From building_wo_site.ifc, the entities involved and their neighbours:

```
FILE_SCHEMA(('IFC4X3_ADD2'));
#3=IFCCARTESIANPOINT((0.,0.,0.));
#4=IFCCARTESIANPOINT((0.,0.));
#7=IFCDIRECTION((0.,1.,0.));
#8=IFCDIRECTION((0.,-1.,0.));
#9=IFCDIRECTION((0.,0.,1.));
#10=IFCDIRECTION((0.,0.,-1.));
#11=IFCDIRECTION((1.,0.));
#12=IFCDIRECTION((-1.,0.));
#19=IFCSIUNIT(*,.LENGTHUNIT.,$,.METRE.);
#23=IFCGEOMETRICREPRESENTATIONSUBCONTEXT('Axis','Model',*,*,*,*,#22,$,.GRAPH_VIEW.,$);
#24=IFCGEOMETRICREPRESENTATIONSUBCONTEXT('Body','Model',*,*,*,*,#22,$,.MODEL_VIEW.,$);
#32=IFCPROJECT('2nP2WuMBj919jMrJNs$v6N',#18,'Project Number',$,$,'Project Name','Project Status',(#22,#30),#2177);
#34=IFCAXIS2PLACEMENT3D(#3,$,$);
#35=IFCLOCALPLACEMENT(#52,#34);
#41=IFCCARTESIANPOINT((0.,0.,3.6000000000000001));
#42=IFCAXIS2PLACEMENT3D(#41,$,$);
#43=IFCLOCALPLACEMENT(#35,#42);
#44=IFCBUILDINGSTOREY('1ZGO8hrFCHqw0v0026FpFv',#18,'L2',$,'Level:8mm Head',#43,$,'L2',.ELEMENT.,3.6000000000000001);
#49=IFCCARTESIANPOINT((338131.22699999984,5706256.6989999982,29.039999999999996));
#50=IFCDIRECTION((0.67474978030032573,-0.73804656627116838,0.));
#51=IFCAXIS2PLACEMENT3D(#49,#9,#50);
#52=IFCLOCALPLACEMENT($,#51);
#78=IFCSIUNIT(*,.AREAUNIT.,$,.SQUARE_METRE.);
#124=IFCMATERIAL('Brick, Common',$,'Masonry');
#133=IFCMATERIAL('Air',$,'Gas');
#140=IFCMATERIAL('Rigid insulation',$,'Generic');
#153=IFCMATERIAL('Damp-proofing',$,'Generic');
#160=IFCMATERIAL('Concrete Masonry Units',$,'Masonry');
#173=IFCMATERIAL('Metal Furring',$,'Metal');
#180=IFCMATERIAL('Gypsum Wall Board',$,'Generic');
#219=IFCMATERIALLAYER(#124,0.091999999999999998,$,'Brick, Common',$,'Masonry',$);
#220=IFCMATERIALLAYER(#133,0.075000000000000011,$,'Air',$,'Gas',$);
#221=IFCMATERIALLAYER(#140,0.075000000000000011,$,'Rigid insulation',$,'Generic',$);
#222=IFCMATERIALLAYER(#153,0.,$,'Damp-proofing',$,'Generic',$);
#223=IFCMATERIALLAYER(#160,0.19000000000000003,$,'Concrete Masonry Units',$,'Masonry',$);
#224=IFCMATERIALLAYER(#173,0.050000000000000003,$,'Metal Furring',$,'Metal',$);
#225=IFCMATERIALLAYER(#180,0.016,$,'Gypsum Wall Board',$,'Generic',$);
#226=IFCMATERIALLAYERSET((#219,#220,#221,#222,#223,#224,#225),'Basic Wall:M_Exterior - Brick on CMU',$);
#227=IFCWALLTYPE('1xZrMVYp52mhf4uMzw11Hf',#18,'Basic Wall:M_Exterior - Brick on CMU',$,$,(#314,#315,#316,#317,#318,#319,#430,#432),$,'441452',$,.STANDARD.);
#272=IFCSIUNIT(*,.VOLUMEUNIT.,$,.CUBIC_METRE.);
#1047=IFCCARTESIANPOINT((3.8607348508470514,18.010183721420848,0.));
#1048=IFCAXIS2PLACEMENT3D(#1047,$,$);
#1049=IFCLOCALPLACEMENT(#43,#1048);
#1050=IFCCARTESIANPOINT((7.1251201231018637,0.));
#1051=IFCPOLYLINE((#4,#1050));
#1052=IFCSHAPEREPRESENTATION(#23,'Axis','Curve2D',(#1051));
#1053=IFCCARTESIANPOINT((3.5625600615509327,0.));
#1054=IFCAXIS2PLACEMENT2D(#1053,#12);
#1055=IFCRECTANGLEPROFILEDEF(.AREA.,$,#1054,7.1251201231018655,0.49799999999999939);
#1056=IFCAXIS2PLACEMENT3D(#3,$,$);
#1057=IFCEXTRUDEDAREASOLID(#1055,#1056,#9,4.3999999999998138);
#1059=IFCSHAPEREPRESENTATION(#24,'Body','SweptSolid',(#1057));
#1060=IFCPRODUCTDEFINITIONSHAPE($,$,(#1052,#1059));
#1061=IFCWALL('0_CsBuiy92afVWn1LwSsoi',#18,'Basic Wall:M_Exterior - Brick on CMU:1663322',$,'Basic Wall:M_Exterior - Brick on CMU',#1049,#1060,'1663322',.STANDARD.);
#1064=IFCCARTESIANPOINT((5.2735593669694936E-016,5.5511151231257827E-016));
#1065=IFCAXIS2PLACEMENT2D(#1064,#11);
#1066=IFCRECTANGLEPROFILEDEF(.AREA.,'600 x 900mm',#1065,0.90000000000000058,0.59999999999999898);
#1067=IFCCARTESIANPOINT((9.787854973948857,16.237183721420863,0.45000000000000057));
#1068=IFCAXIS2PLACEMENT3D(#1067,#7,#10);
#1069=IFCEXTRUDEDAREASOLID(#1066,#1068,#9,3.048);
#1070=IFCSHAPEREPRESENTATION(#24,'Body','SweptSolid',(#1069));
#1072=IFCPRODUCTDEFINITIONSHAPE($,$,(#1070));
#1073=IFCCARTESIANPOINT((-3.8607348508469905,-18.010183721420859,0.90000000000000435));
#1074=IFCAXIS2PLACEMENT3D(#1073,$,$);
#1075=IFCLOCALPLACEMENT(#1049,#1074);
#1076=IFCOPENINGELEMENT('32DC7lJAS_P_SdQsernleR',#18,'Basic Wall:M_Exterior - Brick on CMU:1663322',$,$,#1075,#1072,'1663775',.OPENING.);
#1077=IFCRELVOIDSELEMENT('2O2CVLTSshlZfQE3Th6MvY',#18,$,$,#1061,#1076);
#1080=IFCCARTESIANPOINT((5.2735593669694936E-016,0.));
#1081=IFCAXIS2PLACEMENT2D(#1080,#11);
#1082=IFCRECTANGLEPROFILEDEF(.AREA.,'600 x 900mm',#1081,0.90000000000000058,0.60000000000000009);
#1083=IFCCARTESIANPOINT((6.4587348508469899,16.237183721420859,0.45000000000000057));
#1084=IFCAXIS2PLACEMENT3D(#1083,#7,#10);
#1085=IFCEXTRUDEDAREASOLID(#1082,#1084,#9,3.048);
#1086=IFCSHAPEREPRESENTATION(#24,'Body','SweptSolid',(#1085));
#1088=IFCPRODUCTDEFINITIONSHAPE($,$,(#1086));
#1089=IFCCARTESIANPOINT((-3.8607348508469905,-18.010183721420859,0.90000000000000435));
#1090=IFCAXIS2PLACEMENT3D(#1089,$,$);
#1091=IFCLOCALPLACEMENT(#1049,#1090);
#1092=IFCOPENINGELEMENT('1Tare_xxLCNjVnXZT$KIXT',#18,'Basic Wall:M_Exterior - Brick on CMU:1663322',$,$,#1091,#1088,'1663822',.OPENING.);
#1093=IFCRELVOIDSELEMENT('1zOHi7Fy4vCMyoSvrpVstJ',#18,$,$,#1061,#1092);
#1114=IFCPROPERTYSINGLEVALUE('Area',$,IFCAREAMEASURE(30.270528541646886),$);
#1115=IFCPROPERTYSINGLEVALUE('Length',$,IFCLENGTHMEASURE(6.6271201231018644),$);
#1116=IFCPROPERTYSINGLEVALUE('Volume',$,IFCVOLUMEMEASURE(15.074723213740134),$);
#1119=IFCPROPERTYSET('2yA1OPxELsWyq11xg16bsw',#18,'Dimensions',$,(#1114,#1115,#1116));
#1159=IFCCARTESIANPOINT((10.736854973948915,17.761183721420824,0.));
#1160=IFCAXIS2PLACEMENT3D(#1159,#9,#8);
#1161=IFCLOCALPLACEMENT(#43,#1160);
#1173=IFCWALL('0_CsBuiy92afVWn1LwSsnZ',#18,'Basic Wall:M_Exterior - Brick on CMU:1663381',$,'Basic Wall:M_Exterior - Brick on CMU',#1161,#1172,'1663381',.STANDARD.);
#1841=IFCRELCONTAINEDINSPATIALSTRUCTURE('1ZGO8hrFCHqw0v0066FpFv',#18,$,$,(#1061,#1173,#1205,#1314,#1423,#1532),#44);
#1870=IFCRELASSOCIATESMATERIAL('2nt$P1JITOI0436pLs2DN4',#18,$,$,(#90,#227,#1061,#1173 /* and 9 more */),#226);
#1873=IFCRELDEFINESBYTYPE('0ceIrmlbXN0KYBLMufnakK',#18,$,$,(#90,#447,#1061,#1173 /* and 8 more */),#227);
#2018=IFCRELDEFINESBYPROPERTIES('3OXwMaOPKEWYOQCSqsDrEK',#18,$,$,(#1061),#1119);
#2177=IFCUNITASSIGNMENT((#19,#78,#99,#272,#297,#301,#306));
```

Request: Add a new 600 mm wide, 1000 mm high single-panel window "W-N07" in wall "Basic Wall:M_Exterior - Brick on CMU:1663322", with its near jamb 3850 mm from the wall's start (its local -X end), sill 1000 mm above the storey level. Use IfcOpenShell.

```python
import numpy as np
import ifcopenshell
import ifcopenshell.api.feature
import ifcopenshell.api.geometry
import ifcopenshell.api.pset
import ifcopenshell.api.root
import ifcopenshell.api.spatial
import ifcopenshell.geom
import ifcopenshell.util.element
import ifcopenshell.util.placement
import ifcopenshell.util.representation
import ifcopenshell.util.shape
import ifcopenshell.util.unit

model = ifcopenshell.open("building_wo_site.ifc")
unit_scale = ifcopenshell.util.unit.calculate_unit_scale(model)
area_scale = ifcopenshell.util.unit.calculate_unit_scale(model, "AREAUNIT")
volume_scale = ifcopenshell.util.unit.calculate_unit_scale(model, "VOLUMEUNIT")
settings = ifcopenshell.geom.settings()


def volume(element):
    """Net volume in cubic metres, openings subtracted."""
    shape = ifcopenshell.geom.create_shape(settings, element)
    return ifcopenshell.util.shape.get_volume(shape.geometry)


wall = model.by_id(1061)
storey = ifcopenshell.util.element.get_container(wall, ifc_class="IfcBuildingStorey")
context = ifcopenshell.util.representation.get_context(model, "Model", "Body", "MODEL_VIEW")
before = volume(wall)

width, height, from_end, sill = 0.6, 1, 3.85, 1  # metres

# The wall runs along its own X axis, and the end named is its -X end.
wall_shape = ifcopenshell.geom.create_shape(settings, wall)
x, y, z = ifcopenshell.util.shape.get_vertices(wall_shape.geometry).T
start = x.min() + from_end
face, thickness = float(y.min()), float(y.max() - y.min())
wall_matrix = ifcopenshell.util.placement.get_local_placement(wall.ObjectPlacement)
level = ifcopenshell.util.placement.get_local_placement(storey.ObjectPlacement)[2, 3]


def in_wall(x, y):
    """Placement at x, y metres in the wall's axes, at sill height."""
    matrix = wall_matrix.copy()
    matrix[:, 3] = wall_matrix @ np.array([x / unit_scale, y / unit_scale, 0.0, 1.0])
    matrix[2, 3] = level + sill / unit_scale
    return matrix


# Opening: a box that overshoots both wall faces by 50 mm.
opening = ifcopenshell.api.root.create_entity(model, ifc_class="IfcOpeningElement", predefined_type="OPENING")
box = ifcopenshell.api.geometry.add_wall_representation(
    model, context=context, length=width, height=height, thickness=thickness + 0.1
)
ifcopenshell.api.geometry.assign_representation(model, product=opening, representation=box)
ifcopenshell.api.geometry.edit_object_placement(model, product=opening, matrix=in_wall(start, face - 0.05), is_si=False)
ifcopenshell.api.feature.add_feature(model, feature=opening, element=wall)

window = ifcopenshell.api.root.create_entity(model, ifc_class="IfcWindow", name="W-N07", predefined_type="WINDOW")
window.OverallWidth, window.OverallHeight = width / unit_scale, height / unit_scale
window.PartitioningType = "SINGLE_PANEL"
body = ifcopenshell.api.geometry.add_window_representation(
    model,
    context=context,
    overall_width=window.OverallWidth,
    overall_height=window.OverallHeight,
    partition_type="SINGLE_PANEL",
)
ifcopenshell.api.geometry.assign_representation(model, product=window, representation=body)
ifcopenshell.api.spatial.assign_container(model, products=[window], relating_structure=storey)
ifcopenshell.api.feature.add_filling(model, opening=opening, element=window)

# Centre the window in the wall's thickness.
ifcopenshell.api.geometry.edit_object_placement(model, product=window, matrix=in_wall(start, face), is_si=False)
window_shape = ifcopenshell.geom.create_shape(settings, window)
depth = ifcopenshell.util.shape.get_vertices(window_shape.geometry)[:, 1]
offset = face + thickness / 2 - (depth.min() + depth.max()) / 2
ifcopenshell.api.geometry.edit_object_placement(model, product=window, matrix=in_wall(start, offset), is_si=False)

after = volume(wall)

# Update the wall's stored quantities.
pset = model.by_id(ifcopenshell.util.element.get_pset(wall, "Dimensions", should_inherit=False)["id"])
ifcopenshell.api.pset.edit_pset(model, pset=pset, properties={
    "Area": model.create_entity("IfcAreaMeasure", after / thickness / area_scale),
    "Volume": model.create_entity("IfcVolumeMeasure", after / volume_scale),
})

print(f"wall volume {before:.3f} -> {after:.3f} m3")

model.write("building_wo_site_rev.ifc")
```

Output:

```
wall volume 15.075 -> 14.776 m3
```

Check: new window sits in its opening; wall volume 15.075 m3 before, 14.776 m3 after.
